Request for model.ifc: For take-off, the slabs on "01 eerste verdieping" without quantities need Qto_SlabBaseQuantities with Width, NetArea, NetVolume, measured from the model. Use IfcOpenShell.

First a look at what the model holds.

```python
import ifcopenshell
import ifcopenshell.util.element
import ifcopenshell.util.unit

model = ifcopenshell.open("model.ifc")
print(model.schema)
for unit_type in ("LENGTHUNIT", "AREAUNIT", "VOLUMEUNIT"):
    print(unit_type, ifcopenshell.util.unit.calculate_unit_scale(model, unit_type))
storey = next(s for s in model.by_type("IfcBuildingStorey") if s.Name == "01 eerste verdieping")
slabs = [e for e in ifcopenshell.util.element.get_decomposition(storey) if e.is_a("IfcSlab")]
for e in sorted(slabs, key=lambda e: e.id()):
    print(e.id(), e.is_a(), e.Name, list(ifcopenshell.util.element.get_psets(e, qtos_only=True)), sep=" | ")
```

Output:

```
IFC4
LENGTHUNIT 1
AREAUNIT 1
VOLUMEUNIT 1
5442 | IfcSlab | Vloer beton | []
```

```python
import ifcopenshell
import ifcopenshell.api.pset
import ifcopenshell.geom
import ifcopenshell.util.element
import ifcopenshell.util.shape
import ifcopenshell.util.unit

model = ifcopenshell.open("model.ifc")
unit_scale = ifcopenshell.util.unit.calculate_unit_scale(model)
area_scale = ifcopenshell.util.unit.calculate_unit_scale(model, "AREAUNIT")
volume_scale = ifcopenshell.util.unit.calculate_unit_scale(model, "VOLUMEUNIT")
settings = ifcopenshell.geom.settings()

storey = next(s for s in model.by_type("IfcBuildingStorey") if s.Name == "01 eerste verdieping")
slabs = [e for e in ifcopenshell.util.element.get_decomposition(storey) if e.is_a("IfcSlab")]

for e in sorted(slabs, key=lambda e: e.id()):
    if ifcopenshell.util.element.get_psets(e, qtos_only=True, should_inherit=False):
        continue
    # Geometry comes back in metres, in the element's own axes.
    shape = ifcopenshell.geom.create_shape(settings, e)
    values = {
        "Width": ifcopenshell.util.shape.get_z(shape.geometry) / unit_scale,
        "NetArea": ifcopenshell.util.shape.get_footprint_area(shape.geometry) / area_scale,
        "NetVolume": ifcopenshell.util.shape.get_volume(shape.geometry) / volume_scale,
    }
    qto = ifcopenshell.api.pset.add_qto(model, product=e, name="Qto_SlabBaseQuantities")
    ifcopenshell.api.pset.edit_qto(model, qto=qto, properties=values)
    print(e.id(), {k: round(v, 3) for k, v in values.items()})

model.write("model-out.ifc")
```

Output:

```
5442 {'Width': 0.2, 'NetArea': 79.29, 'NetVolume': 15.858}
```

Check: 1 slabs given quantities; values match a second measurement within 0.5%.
